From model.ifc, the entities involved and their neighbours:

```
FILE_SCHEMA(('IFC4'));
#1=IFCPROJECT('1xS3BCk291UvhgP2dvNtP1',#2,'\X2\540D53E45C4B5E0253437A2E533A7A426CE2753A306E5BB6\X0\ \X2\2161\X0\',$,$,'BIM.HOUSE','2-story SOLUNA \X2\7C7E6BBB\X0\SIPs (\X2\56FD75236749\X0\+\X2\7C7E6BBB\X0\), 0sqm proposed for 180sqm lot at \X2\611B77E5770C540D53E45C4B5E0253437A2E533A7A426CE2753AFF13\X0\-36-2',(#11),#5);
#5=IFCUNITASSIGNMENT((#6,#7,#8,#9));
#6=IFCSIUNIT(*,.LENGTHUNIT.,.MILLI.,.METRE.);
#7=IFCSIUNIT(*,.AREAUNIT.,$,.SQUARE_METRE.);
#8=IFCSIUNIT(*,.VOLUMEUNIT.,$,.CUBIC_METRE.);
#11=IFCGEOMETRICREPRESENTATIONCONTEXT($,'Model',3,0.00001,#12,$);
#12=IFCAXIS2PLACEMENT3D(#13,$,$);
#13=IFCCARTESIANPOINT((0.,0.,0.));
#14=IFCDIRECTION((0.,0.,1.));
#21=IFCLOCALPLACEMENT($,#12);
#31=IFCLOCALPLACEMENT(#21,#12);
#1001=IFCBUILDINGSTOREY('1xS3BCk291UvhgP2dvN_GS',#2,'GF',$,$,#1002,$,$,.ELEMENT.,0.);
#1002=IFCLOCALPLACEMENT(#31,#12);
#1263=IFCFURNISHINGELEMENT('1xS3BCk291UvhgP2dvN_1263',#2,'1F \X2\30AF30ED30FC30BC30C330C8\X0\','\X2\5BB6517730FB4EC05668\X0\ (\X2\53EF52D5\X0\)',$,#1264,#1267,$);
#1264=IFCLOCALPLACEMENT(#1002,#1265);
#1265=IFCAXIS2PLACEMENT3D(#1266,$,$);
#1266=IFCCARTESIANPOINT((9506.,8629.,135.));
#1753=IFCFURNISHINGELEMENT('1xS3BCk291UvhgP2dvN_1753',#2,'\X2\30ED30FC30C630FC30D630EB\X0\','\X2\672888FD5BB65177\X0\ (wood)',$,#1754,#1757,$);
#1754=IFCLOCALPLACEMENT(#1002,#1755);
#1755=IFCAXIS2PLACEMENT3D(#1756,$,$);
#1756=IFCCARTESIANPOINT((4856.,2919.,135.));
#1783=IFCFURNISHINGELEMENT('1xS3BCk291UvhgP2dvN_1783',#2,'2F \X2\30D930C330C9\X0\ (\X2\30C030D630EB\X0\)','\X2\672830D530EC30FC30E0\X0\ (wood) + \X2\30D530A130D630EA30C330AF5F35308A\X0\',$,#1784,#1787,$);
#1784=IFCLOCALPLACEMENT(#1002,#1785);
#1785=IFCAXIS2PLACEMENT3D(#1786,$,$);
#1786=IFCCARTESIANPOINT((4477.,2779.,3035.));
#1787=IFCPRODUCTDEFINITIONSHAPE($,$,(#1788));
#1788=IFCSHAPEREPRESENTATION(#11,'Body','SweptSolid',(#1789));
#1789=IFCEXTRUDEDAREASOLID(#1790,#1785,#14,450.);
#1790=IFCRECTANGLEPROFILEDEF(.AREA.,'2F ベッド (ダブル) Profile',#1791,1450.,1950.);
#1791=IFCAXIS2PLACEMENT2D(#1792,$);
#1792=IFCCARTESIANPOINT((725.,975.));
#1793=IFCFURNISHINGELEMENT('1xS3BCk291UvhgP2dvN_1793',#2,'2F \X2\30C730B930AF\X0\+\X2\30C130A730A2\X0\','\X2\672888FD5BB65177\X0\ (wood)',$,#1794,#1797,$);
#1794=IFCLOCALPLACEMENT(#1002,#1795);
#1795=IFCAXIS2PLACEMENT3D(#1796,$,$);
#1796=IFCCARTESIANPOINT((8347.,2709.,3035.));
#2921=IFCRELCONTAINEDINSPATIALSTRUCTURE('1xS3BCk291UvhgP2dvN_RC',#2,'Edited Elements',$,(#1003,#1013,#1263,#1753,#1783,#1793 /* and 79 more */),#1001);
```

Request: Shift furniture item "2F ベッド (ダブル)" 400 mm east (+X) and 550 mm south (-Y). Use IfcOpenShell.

```python
import ifcopenshell
import ifcopenshell.api.geometry
import ifcopenshell.util.placement
import ifcopenshell.util.unit

model = ifcopenshell.open("model.ifc")
unit_scale = ifcopenshell.util.unit.calculate_unit_scale(model)

item = model.by_guid("1xS3BCk291UvhgP2dvN_1783")
matrix = ifcopenshell.util.placement.get_local_placement(item.ObjectPlacement)
matrix[0, 3] += 0.4 / unit_scale
matrix[1, 3] -= 0.55 / unit_scale
ifcopenshell.api.geometry.edit_object_placement(model, product=item, matrix=matrix, is_si=False)

print(ifcopenshell.util.placement.get_local_placement(item.ObjectPlacement).round(3) + 0.0)

model.write("model-out.ifc")
```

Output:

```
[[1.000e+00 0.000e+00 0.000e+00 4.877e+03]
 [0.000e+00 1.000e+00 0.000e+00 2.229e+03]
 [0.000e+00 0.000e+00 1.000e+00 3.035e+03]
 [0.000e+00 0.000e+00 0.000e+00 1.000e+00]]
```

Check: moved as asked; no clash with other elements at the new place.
